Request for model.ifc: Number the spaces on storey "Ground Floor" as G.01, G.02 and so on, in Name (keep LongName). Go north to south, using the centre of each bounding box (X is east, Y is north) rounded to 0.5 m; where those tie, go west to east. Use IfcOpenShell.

First a look at what the model holds.

```python
import ifcopenshell
import ifcopenshell.util.element
import ifcopenshell.util.placement

model = ifcopenshell.open("model.ifc")
print(model.schema)
storey = next(s for s in model.by_type("IfcBuildingStorey") if s.Name == "Ground Floor")
spaces = [e for e in ifcopenshell.util.element.get_decomposition(storey) if e.is_a("IfcSpace")]
for e in sorted(spaces, key=lambda e: e.id()):
    origin = ifcopenshell.util.placement.get_local_placement(e.ObjectPlacement)[:3, 3]
    print(e.id(), e.Name, e.LongName, origin.round(2) + 0.0, sep=" | ")
```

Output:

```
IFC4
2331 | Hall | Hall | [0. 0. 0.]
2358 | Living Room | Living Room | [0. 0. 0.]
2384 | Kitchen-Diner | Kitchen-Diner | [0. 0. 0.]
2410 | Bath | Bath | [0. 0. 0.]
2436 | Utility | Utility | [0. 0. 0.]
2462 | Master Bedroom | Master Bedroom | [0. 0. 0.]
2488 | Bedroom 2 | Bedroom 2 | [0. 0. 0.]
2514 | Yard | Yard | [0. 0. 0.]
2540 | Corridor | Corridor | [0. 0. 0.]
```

```python
import ifcopenshell
import ifcopenshell.geom
import ifcopenshell.util.element
import ifcopenshell.util.shape

model = ifcopenshell.open("model.ifc")
settings = ifcopenshell.geom.settings()
settings.set("use-world-coords", True)


def centre(element):
    shape = ifcopenshell.geom.create_shape(settings, element)
    return ifcopenshell.util.shape.get_bbox_centroid(shape.geometry)


storey = next(s for s in model.by_type("IfcBuildingStorey") if s.Name == "Ground Floor")
spaces = [e for e in ifcopenshell.util.element.get_decomposition(storey) if e.is_a("IfcSpace")]

# Insertion points can sit at a corner or the storey origin, so sort by the geometry (in metres).
centres = {e: centre(e) for e in spaces}
spaces.sort(key=lambda e: (-round(centres[e][1] / 0.5), centres[e][0]))

for i, e in enumerate(spaces, start=1):
    number = f"G.{i:02d}"
    e.Name = number
    print(e.id(), number)

model.write("model_edited.ifc")
```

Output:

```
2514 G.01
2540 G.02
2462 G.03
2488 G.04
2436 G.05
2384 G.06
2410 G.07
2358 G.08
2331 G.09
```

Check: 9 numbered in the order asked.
